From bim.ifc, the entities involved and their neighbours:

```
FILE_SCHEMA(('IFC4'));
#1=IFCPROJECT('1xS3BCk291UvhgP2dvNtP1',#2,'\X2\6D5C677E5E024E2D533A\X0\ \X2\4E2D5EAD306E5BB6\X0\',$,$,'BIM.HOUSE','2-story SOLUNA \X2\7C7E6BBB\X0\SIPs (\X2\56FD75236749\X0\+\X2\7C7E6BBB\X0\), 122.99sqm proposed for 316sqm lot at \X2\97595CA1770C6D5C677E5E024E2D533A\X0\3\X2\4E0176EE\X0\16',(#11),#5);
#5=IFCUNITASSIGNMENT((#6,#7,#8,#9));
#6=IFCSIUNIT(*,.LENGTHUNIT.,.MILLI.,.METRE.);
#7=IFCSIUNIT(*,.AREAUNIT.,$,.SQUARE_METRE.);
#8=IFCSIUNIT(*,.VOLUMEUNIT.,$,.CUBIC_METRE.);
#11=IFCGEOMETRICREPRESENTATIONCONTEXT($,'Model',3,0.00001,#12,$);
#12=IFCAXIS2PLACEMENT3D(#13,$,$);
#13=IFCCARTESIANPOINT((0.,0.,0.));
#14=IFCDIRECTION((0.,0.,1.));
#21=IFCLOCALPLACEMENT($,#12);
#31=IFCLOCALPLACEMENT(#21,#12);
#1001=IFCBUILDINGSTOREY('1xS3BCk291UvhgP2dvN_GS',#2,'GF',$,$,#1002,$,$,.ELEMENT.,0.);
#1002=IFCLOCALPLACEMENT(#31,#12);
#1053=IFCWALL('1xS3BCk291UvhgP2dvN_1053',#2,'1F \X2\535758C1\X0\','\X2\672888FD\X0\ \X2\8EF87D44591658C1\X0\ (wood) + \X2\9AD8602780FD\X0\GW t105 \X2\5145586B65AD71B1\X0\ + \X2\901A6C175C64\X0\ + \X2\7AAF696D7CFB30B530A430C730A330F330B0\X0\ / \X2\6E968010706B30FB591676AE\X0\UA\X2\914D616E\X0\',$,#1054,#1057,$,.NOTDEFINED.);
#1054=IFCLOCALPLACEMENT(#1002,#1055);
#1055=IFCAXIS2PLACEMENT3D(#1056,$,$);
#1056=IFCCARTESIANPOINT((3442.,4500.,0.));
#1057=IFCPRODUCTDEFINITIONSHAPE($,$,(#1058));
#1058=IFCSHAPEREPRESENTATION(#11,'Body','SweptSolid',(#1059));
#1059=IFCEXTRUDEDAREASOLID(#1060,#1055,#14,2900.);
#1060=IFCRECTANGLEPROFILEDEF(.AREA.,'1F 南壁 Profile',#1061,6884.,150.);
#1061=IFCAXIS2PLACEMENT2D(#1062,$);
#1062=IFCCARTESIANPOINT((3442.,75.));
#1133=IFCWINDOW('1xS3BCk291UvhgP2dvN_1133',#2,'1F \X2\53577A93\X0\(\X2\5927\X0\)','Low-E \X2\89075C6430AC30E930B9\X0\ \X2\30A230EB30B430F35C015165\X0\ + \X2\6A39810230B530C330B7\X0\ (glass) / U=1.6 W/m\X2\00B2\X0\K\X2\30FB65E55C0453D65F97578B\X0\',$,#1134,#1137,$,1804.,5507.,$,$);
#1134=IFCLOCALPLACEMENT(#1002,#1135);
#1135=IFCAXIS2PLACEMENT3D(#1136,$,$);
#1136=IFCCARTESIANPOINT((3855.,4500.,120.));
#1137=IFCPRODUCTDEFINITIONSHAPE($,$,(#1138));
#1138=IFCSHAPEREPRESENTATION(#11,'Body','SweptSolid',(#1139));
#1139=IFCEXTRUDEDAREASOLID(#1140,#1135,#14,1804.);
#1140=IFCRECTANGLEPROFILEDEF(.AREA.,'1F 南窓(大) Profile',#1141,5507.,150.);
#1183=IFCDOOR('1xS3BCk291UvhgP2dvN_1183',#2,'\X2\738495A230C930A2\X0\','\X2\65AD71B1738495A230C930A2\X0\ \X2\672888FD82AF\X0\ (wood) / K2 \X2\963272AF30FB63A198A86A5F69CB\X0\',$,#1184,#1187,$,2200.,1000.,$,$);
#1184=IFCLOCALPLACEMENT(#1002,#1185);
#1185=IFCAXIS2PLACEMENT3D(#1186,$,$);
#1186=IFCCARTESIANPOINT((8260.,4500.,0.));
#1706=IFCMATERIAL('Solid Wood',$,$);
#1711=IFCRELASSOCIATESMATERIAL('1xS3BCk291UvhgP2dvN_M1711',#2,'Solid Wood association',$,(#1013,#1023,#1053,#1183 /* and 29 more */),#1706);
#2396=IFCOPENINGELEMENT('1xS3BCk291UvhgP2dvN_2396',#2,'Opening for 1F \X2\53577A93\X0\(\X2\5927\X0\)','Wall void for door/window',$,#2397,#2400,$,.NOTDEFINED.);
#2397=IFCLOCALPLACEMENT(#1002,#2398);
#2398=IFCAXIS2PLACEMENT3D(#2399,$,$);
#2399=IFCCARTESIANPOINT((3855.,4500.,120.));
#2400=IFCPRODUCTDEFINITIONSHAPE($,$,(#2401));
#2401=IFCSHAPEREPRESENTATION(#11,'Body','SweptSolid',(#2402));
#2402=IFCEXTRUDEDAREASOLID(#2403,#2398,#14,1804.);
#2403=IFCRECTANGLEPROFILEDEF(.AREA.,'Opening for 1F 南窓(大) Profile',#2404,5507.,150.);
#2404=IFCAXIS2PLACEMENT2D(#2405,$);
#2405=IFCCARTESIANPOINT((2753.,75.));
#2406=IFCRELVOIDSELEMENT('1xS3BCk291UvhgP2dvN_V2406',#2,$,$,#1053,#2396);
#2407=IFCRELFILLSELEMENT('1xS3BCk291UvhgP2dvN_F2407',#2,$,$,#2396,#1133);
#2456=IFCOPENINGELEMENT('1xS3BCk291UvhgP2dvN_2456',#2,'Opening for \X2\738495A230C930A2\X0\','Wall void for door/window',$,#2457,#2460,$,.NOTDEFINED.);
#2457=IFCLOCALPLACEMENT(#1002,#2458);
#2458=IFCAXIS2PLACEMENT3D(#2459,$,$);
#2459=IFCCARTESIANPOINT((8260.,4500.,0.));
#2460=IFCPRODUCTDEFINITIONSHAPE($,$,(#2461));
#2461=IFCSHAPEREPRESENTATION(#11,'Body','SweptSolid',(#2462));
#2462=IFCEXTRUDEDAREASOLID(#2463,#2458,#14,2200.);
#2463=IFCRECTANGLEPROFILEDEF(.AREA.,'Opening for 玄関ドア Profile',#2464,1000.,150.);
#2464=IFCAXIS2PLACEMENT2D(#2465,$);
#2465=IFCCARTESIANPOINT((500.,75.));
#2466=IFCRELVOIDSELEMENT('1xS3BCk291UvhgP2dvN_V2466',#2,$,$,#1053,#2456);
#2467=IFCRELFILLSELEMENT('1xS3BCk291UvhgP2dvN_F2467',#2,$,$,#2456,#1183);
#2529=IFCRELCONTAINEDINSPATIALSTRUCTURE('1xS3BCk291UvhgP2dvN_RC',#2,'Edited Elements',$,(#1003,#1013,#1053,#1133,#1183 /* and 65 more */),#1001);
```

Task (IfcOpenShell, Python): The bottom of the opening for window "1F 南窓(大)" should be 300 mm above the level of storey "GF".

```python
import numpy as np
import ifcopenshell
import ifcopenshell.api.geometry
import ifcopenshell.geom
import ifcopenshell.util.element
import ifcopenshell.util.placement
import ifcopenshell.util.shape
import ifcopenshell.util.unit

model = ifcopenshell.open("bim.ifc")
unit_scale = ifcopenshell.util.unit.calculate_unit_scale(model)

window = model.by_id(1133)
opening = window.FillsVoids[0].RelatingOpeningElement
storey = ifcopenshell.util.element.get_container(window, ifc_class="IfcBuildingStorey")
level = ifcopenshell.util.placement.get_local_placement(storey.ObjectPlacement)[2, 3]

# The opening's origin need not be at the sill, so measure its lowest point.
shape = ifcopenshell.geom.create_shape(ifcopenshell.geom.settings(), opening)
bottom = ifcopenshell.util.shape.get_shape_bottom_elevation(shape, shape.geometry) / unit_scale
dz = level + 0.3 / unit_scale - bottom

shift = np.array([0.0, 0.0, dz])
# The window is not placed relative to its opening, so move both.
for product in (opening, window):
    matrix = ifcopenshell.util.placement.get_local_placement(product.ObjectPlacement)
    matrix[:3, 3] += shift
    ifcopenshell.api.geometry.edit_object_placement(model, product=product, matrix=matrix, is_si=False)

print(f"moved by {dz * unit_scale:+.3f} m")

model.write("bim_edited.ifc")
```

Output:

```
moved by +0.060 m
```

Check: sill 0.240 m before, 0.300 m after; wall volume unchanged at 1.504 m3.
